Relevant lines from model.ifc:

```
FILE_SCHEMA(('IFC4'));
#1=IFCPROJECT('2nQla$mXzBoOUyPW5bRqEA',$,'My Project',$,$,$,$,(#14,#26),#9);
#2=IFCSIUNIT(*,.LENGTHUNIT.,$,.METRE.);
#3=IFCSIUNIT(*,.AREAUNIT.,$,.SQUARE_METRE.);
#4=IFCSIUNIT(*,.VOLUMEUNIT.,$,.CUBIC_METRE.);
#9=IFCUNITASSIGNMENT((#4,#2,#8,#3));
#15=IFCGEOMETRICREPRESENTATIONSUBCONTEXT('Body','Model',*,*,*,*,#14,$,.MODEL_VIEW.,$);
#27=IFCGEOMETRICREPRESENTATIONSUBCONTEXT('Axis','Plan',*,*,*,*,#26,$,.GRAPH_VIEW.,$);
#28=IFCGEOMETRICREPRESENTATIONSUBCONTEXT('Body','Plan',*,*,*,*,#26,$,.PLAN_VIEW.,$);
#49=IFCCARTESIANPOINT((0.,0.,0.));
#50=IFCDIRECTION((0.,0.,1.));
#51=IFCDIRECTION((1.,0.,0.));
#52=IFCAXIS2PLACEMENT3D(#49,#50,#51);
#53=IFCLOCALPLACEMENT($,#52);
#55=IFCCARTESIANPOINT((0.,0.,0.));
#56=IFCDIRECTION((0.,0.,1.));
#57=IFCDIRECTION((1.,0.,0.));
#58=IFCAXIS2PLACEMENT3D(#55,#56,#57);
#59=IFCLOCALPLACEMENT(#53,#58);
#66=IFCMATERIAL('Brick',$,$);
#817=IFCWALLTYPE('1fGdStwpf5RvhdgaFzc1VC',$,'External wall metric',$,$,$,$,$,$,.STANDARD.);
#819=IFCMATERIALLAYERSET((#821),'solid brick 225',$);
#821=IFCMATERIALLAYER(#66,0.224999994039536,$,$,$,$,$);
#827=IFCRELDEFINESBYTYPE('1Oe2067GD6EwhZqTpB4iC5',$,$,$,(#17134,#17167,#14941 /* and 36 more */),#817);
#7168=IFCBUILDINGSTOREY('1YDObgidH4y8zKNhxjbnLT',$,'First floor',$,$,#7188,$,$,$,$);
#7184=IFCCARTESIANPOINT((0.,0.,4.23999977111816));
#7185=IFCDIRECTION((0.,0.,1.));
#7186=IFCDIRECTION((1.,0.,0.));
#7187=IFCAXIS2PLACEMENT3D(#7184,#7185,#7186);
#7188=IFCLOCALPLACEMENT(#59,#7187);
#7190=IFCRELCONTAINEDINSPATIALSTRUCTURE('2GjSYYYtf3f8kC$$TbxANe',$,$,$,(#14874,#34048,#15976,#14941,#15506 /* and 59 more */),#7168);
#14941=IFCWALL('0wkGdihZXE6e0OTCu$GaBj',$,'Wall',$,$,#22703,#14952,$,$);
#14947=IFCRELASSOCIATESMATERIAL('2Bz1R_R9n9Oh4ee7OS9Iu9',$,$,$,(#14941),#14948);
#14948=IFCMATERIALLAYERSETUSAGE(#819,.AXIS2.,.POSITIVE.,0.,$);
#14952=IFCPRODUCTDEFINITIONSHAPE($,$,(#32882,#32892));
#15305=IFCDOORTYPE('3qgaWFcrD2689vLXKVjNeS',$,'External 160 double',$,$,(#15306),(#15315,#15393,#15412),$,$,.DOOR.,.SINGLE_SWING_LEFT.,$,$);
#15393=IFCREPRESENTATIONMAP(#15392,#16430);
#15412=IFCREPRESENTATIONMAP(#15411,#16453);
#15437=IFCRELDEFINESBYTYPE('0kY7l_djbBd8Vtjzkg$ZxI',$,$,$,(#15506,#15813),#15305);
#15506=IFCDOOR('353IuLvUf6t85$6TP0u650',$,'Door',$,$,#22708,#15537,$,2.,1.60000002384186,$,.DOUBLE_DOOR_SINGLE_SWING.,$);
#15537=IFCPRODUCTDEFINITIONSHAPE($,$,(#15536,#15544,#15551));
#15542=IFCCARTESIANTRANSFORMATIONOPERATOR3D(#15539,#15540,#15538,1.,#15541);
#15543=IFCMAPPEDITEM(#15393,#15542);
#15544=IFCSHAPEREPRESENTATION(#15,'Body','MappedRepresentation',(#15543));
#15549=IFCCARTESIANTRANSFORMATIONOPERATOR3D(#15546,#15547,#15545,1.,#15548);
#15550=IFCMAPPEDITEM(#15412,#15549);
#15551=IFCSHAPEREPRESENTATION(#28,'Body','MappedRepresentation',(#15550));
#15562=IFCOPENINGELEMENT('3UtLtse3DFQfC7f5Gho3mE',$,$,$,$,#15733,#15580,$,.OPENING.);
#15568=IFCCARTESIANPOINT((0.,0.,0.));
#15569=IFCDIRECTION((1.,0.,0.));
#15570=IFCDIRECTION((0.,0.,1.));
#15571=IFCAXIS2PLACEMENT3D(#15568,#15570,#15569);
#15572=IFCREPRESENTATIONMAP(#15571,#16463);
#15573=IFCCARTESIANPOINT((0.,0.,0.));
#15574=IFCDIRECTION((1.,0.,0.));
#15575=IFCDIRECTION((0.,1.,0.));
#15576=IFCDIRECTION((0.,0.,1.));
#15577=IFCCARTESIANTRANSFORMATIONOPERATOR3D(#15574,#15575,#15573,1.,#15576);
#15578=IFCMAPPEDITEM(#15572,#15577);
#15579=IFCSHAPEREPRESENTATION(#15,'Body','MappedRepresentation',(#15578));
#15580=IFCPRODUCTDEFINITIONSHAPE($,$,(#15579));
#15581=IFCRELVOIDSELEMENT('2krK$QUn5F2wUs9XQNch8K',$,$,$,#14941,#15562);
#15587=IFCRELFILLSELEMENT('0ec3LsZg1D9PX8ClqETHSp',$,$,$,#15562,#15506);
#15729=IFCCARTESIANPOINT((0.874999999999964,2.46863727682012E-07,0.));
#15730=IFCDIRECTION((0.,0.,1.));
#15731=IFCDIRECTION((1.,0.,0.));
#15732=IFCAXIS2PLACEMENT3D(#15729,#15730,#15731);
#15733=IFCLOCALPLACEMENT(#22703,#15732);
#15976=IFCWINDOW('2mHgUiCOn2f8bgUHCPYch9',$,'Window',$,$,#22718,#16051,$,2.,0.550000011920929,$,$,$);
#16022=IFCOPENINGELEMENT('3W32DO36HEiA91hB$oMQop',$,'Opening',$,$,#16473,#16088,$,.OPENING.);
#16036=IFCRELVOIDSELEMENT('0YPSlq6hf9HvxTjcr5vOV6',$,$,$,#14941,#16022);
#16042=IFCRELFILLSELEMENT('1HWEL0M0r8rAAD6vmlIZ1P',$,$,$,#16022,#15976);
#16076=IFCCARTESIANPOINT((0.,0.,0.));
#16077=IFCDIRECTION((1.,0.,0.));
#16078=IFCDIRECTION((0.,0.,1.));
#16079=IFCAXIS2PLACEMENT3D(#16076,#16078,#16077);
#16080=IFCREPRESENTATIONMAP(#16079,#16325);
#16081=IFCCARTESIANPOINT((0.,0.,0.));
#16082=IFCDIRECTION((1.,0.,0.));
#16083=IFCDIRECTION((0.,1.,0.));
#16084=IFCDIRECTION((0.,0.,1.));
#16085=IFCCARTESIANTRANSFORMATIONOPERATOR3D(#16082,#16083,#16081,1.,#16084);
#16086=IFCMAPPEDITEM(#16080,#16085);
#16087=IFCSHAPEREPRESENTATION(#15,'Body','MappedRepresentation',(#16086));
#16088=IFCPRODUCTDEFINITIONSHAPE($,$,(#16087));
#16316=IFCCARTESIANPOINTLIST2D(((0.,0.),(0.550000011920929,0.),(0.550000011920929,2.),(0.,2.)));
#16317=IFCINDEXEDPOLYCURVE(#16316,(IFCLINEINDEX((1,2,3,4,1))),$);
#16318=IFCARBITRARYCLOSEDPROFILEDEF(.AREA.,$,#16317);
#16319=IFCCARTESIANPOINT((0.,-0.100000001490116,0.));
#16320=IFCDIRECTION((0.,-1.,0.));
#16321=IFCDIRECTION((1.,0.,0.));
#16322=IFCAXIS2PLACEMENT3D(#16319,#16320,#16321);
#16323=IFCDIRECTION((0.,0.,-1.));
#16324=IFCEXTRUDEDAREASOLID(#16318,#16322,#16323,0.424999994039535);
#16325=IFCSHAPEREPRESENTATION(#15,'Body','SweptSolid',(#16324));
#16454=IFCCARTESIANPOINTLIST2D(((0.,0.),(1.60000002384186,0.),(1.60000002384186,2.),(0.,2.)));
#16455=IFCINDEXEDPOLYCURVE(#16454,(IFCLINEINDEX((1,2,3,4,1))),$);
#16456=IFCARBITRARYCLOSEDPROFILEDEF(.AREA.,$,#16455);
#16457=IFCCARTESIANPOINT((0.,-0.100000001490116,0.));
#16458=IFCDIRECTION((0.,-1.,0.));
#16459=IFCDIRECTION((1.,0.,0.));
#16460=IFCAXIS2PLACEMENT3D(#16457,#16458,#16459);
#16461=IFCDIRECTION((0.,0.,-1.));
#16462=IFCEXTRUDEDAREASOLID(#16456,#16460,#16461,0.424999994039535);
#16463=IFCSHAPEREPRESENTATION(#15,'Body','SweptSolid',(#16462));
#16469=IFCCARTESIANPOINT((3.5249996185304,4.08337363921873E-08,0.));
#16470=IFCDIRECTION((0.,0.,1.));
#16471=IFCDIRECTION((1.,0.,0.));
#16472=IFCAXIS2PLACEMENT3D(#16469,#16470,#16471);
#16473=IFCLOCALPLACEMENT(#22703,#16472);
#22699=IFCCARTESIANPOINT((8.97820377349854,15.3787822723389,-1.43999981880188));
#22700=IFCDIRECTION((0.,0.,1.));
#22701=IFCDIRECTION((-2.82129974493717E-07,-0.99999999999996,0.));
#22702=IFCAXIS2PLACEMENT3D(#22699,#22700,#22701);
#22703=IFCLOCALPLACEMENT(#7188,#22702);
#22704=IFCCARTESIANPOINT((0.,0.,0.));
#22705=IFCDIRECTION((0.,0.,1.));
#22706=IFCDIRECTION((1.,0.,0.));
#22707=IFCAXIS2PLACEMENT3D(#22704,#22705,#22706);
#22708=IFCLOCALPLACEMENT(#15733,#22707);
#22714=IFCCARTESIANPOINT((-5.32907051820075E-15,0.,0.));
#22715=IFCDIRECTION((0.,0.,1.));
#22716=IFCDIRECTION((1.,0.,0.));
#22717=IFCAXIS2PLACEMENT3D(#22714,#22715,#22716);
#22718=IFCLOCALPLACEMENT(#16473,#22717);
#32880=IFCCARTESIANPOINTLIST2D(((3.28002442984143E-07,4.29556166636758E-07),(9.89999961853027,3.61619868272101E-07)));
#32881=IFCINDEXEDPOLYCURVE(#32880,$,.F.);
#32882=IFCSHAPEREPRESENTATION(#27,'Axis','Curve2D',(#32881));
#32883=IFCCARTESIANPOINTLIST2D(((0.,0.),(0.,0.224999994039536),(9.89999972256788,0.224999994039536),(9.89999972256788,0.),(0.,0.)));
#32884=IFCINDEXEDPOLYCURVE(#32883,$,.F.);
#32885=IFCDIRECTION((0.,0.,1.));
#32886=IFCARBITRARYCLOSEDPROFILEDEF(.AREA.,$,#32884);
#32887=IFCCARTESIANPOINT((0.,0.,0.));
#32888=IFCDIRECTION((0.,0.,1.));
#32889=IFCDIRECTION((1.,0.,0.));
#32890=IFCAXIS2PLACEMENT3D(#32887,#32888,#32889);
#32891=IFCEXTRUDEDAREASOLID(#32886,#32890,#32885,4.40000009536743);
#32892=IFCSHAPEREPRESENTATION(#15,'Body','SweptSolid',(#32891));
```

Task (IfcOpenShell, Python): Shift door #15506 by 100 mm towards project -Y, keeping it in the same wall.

```python
import ifcopenshell
import ifcopenshell.api.geometry
import ifcopenshell.util.placement
import ifcopenshell.util.unit

model = ifcopenshell.open("model.ifc")
unit_scale = ifcopenshell.util.unit.calculate_unit_scale(model)

door = model.by_id(15506)
opening = door.FillsVoids[0].RelatingOpeningElement
wall = opening.VoidsElements[0].RelatingBuildingElement

wall_matrix = ifcopenshell.util.placement.get_local_placement(wall.ObjectPlacement)
shift = wall_matrix[:3, 0] * 0.1 / unit_scale
before = ifcopenshell.util.placement.get_local_placement(door.ObjectPlacement)[:3, 3].copy()

# The door is placed relative to its opening, so it follows when the opening moves.
matrix = ifcopenshell.util.placement.get_local_placement(opening.ObjectPlacement)
matrix[:3, 3] += shift
ifcopenshell.api.geometry.edit_object_placement(
    model, product=opening, matrix=matrix, is_si=False, should_transform_children=True
)

after = ifcopenshell.util.placement.get_local_placement(door.ObjectPlacement)[:3, 3]
print("door moved by", (after - before).round(3) + 0.0)

model.write("model_rev.ifc")
```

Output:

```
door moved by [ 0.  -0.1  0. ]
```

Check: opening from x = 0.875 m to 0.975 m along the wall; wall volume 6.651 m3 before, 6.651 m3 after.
